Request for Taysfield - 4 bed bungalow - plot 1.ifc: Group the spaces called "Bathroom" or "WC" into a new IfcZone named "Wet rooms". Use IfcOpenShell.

First a look at what the model holds.

```python
import ifcopenshell

model = ifcopenshell.open("Taysfield - 4 bed bungalow - plot 1.ifc")
print(model.schema)
seen = {}
for space in model.by_type("IfcSpace"):
    seen[space.LongName] = seen.get(space.LongName, 0) + 1
for name, count in sorted(seen.items(), key=str):
    print(count, "x", name)
print("zones:", [z.Name for z in model.by_type("IfcZone")][:20])
```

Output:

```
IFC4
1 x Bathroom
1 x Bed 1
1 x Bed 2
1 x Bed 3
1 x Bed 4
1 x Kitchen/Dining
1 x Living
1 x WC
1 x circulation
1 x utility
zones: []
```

```python
import ifcopenshell
import ifcopenshell.api.group
import ifcopenshell.api.root

model = ifcopenshell.open("Taysfield - 4 bed bungalow - plot 1.ifc")

names = {"Bathroom", "WC"}
spaces = [s for s in model.by_type("IfcSpace") if s.LongName in names]

zone = ifcopenshell.api.root.create_entity(model, ifc_class="IfcZone", name="Wet rooms")
ifcopenshell.api.group.assign_group(model, products=spaces, group=zone)
print(len(spaces), "spaces in", zone.Name)

model.write("Taysfield - 4 bed bungalow - plot 1_rev.ifc")
```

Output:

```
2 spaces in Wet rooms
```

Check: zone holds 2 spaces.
